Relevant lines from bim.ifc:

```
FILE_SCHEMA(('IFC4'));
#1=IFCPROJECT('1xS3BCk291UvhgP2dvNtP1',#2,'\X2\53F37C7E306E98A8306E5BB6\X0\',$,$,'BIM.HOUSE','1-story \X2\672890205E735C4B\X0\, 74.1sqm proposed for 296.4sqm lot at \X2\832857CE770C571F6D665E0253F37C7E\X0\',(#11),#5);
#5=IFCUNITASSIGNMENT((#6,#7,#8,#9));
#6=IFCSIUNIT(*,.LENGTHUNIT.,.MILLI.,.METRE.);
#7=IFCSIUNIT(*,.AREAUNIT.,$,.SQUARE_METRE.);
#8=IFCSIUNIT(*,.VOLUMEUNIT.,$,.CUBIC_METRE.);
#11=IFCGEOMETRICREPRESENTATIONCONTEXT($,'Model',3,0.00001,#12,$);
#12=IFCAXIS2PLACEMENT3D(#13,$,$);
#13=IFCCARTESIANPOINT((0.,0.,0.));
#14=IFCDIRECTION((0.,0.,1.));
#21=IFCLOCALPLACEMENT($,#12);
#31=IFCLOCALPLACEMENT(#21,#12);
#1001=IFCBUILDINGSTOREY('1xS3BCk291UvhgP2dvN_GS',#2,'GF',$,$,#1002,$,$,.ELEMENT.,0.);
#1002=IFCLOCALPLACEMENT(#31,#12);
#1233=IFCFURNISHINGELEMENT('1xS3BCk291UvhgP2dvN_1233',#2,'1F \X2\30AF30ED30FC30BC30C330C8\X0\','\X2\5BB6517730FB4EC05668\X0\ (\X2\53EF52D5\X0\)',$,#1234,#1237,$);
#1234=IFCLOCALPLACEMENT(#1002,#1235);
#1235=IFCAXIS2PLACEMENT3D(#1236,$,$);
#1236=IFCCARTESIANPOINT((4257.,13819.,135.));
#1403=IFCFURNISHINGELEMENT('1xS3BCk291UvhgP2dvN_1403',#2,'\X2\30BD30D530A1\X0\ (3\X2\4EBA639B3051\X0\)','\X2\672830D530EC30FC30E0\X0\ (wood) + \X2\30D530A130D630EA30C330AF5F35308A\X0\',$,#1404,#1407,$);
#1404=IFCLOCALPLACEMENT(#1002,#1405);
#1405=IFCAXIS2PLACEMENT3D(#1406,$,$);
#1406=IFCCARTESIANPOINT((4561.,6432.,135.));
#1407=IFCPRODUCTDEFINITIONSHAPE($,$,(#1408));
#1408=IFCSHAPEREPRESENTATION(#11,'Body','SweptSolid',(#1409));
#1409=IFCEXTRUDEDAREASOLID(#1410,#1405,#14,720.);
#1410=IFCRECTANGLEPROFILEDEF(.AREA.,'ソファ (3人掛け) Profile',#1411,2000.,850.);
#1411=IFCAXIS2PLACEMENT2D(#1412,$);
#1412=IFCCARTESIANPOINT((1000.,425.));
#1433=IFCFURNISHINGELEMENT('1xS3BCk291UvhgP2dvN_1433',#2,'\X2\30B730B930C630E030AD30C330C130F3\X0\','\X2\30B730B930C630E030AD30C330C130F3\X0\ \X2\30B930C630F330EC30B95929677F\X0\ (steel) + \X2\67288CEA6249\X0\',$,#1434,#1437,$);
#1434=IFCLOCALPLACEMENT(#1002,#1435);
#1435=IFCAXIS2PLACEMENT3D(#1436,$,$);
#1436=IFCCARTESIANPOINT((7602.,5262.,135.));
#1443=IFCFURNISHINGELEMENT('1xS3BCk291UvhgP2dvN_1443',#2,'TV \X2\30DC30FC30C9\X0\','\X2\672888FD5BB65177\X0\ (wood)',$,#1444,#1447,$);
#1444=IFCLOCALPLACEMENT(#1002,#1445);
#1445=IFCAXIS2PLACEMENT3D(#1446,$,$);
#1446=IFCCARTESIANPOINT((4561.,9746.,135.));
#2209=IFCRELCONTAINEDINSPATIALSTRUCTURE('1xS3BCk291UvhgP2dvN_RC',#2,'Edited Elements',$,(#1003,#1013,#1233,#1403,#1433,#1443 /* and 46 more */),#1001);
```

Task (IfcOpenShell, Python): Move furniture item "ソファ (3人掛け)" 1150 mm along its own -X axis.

```python
import ifcopenshell
import ifcopenshell.api.geometry
import ifcopenshell.util.placement

model = ifcopenshell.open("bim.ifc")

item = model.by_guid("1xS3BCk291UvhgP2dvN_1403")
matrix = ifcopenshell.util.placement.get_local_placement(item.ObjectPlacement)
matrix[:3, 3] -= matrix[:3, 0] * 1150.0
ifcopenshell.api.geometry.edit_object_placement(model, product=item, matrix=matrix, is_si=False)

print(ifcopenshell.util.placement.get_local_placement(item.ObjectPlacement).round(3) + 0.0)

model.write("bim_v2.ifc")
```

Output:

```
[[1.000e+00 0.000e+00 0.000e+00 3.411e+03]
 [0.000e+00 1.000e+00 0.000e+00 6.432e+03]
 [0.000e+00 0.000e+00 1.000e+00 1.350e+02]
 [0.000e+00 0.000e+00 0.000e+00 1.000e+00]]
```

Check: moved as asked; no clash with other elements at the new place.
